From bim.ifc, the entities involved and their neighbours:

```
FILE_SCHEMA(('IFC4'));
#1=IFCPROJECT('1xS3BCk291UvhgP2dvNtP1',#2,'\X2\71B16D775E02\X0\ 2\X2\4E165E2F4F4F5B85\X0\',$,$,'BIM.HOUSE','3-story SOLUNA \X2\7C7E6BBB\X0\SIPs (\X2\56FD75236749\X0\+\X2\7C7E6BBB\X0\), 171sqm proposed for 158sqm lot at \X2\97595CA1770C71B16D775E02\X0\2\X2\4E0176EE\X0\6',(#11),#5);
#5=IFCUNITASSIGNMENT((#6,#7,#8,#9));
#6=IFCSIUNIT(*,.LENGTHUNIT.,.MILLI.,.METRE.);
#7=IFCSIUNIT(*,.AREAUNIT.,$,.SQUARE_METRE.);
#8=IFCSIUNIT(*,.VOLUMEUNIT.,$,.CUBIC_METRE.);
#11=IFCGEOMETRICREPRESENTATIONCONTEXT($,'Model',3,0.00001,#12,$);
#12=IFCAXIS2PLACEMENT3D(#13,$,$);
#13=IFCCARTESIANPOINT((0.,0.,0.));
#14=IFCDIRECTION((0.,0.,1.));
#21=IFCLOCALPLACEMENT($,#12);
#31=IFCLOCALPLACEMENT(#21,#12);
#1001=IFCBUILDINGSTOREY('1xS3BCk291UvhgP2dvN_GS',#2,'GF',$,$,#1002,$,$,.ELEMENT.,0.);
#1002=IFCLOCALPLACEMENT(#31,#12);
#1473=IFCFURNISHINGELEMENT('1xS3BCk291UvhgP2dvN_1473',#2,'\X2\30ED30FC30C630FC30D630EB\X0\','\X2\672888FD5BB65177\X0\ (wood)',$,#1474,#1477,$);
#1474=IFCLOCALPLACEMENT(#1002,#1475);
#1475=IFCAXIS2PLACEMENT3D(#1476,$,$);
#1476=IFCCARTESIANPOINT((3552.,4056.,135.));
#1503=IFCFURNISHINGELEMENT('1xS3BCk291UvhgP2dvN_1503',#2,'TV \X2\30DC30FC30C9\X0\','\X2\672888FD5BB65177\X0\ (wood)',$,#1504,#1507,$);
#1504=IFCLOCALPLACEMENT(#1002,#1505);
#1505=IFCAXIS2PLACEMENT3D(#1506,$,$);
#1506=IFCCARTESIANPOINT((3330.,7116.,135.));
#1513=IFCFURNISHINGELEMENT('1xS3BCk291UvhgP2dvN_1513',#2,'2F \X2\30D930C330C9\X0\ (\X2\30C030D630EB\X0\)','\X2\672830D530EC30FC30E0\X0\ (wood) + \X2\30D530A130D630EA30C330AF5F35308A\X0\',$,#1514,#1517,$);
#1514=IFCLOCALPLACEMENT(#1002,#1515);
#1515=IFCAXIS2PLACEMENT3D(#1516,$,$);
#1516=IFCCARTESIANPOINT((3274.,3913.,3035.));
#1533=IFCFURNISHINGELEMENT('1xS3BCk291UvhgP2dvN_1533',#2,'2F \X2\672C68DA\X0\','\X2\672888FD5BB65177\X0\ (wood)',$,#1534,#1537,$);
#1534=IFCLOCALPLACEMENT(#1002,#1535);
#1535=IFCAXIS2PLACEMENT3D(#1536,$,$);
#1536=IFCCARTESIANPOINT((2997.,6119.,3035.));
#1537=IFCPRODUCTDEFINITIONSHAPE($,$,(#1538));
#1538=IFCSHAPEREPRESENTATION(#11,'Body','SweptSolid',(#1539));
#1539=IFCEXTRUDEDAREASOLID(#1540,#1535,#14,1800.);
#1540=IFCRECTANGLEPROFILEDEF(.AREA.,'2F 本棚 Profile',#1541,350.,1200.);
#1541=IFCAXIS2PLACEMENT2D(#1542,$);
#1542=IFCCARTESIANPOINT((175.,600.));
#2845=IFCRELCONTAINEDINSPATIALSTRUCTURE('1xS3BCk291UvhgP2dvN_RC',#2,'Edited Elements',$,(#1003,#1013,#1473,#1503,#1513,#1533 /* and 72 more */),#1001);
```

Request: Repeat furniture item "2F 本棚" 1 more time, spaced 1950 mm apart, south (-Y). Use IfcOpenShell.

```python
import numpy as np
import ifcopenshell
import ifcopenshell.api.geometry
import ifcopenshell.api.root
import ifcopenshell.util.element
import ifcopenshell.util.placement
import ifcopenshell.util.unit

model = ifcopenshell.open("bim.ifc")
unit_scale = ifcopenshell.util.unit.calculate_unit_scale(model)


def reuse_history(source, copy):
    """copy_class also copies each property set's owner history, people and application; keep the originals."""
    for rel in copy.IsDefinedBy:
        if rel.is_a("IfcRelDefinesByProperties") and (history := rel.RelatingPropertyDefinition.OwnerHistory):
            rel.RelatingPropertyDefinition.OwnerHistory = source.OwnerHistory
            ifcopenshell.util.element.remove_deep2(model, history)


source = model.by_guid("1xS3BCk291UvhgP2dvN_1533")
base = ifcopenshell.util.placement.get_local_placement(source.ObjectPlacement)
step = np.array([0.0, -1.0, 0.0]) * 1.95 / unit_scale

for i in range(1, 2):
    copy = ifcopenshell.api.root.copy_class(model, product=source)
    copy.Representation = ifcopenshell.util.element.copy_deep(
        model, source.Representation, exclude=["IfcGeometricRepresentationContext", "IfcRepresentationMap"]
    )
    reuse_history(source, copy)
    matrix = base.copy()
    matrix[:3, 3] += i * step
    print("added at", matrix[:3, 3].round(3) + 0.0)
    ifcopenshell.api.geometry.edit_object_placement(model, product=copy, matrix=matrix, is_si=False)

model.write("bim_v2.ifc")
```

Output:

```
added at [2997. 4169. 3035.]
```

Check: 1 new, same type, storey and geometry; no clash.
